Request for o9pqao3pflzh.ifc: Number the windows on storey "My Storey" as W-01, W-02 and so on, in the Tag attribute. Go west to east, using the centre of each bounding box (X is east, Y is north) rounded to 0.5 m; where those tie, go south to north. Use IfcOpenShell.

First a look at what the model holds.

```python
import ifcopenshell
import ifcopenshell.util.element
import ifcopenshell.util.placement

model = ifcopenshell.open("o9pqao3pflzh.ifc")
print(model.schema)
storey = next(s for s in model.by_type("IfcBuildingStorey") if s.Name == "My Storey")
windows = [e for e in ifcopenshell.util.element.get_decomposition(storey) if e.is_a("IfcWindow")]
for e in sorted(windows, key=lambda e: e.id()):
    origin = ifcopenshell.util.placement.get_local_placement(e.ObjectPlacement)[:3, 3]
    print(e.id(), e.Tag, e.Name, origin.round(2) + 0.0, sep=" | ")
```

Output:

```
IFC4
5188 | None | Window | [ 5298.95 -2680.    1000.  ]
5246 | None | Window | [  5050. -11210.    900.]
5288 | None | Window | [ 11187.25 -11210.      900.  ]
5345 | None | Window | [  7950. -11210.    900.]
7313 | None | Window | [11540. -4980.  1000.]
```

```python
import ifcopenshell
import ifcopenshell.geom
import ifcopenshell.util.element
import ifcopenshell.util.shape

model = ifcopenshell.open("o9pqao3pflzh.ifc")
settings = ifcopenshell.geom.settings()
settings.set("use-world-coords", True)


def centre(element):
    shape = ifcopenshell.geom.create_shape(settings, element)
    return ifcopenshell.util.shape.get_bbox_centroid(shape.geometry)


storey = next(s for s in model.by_type("IfcBuildingStorey") if s.Name == "My Storey")
windows = [e for e in ifcopenshell.util.element.get_decomposition(storey) if e.is_a("IfcWindow")]

# Insertion points can sit at a corner or the storey origin, so sort by the geometry (in metres).
centres = {e: centre(e) for e in windows}
windows.sort(key=lambda e: (round(centres[e][0] / 0.5), centres[e][1]))

for i, e in enumerate(windows, start=1):
    number = f"W-{i:02d}"
    e.Tag = number
    print(e.id(), number)

model.write("o9pqao3pflzh_v2.ifc")
```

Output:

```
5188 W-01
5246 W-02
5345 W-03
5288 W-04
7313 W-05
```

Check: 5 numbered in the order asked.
